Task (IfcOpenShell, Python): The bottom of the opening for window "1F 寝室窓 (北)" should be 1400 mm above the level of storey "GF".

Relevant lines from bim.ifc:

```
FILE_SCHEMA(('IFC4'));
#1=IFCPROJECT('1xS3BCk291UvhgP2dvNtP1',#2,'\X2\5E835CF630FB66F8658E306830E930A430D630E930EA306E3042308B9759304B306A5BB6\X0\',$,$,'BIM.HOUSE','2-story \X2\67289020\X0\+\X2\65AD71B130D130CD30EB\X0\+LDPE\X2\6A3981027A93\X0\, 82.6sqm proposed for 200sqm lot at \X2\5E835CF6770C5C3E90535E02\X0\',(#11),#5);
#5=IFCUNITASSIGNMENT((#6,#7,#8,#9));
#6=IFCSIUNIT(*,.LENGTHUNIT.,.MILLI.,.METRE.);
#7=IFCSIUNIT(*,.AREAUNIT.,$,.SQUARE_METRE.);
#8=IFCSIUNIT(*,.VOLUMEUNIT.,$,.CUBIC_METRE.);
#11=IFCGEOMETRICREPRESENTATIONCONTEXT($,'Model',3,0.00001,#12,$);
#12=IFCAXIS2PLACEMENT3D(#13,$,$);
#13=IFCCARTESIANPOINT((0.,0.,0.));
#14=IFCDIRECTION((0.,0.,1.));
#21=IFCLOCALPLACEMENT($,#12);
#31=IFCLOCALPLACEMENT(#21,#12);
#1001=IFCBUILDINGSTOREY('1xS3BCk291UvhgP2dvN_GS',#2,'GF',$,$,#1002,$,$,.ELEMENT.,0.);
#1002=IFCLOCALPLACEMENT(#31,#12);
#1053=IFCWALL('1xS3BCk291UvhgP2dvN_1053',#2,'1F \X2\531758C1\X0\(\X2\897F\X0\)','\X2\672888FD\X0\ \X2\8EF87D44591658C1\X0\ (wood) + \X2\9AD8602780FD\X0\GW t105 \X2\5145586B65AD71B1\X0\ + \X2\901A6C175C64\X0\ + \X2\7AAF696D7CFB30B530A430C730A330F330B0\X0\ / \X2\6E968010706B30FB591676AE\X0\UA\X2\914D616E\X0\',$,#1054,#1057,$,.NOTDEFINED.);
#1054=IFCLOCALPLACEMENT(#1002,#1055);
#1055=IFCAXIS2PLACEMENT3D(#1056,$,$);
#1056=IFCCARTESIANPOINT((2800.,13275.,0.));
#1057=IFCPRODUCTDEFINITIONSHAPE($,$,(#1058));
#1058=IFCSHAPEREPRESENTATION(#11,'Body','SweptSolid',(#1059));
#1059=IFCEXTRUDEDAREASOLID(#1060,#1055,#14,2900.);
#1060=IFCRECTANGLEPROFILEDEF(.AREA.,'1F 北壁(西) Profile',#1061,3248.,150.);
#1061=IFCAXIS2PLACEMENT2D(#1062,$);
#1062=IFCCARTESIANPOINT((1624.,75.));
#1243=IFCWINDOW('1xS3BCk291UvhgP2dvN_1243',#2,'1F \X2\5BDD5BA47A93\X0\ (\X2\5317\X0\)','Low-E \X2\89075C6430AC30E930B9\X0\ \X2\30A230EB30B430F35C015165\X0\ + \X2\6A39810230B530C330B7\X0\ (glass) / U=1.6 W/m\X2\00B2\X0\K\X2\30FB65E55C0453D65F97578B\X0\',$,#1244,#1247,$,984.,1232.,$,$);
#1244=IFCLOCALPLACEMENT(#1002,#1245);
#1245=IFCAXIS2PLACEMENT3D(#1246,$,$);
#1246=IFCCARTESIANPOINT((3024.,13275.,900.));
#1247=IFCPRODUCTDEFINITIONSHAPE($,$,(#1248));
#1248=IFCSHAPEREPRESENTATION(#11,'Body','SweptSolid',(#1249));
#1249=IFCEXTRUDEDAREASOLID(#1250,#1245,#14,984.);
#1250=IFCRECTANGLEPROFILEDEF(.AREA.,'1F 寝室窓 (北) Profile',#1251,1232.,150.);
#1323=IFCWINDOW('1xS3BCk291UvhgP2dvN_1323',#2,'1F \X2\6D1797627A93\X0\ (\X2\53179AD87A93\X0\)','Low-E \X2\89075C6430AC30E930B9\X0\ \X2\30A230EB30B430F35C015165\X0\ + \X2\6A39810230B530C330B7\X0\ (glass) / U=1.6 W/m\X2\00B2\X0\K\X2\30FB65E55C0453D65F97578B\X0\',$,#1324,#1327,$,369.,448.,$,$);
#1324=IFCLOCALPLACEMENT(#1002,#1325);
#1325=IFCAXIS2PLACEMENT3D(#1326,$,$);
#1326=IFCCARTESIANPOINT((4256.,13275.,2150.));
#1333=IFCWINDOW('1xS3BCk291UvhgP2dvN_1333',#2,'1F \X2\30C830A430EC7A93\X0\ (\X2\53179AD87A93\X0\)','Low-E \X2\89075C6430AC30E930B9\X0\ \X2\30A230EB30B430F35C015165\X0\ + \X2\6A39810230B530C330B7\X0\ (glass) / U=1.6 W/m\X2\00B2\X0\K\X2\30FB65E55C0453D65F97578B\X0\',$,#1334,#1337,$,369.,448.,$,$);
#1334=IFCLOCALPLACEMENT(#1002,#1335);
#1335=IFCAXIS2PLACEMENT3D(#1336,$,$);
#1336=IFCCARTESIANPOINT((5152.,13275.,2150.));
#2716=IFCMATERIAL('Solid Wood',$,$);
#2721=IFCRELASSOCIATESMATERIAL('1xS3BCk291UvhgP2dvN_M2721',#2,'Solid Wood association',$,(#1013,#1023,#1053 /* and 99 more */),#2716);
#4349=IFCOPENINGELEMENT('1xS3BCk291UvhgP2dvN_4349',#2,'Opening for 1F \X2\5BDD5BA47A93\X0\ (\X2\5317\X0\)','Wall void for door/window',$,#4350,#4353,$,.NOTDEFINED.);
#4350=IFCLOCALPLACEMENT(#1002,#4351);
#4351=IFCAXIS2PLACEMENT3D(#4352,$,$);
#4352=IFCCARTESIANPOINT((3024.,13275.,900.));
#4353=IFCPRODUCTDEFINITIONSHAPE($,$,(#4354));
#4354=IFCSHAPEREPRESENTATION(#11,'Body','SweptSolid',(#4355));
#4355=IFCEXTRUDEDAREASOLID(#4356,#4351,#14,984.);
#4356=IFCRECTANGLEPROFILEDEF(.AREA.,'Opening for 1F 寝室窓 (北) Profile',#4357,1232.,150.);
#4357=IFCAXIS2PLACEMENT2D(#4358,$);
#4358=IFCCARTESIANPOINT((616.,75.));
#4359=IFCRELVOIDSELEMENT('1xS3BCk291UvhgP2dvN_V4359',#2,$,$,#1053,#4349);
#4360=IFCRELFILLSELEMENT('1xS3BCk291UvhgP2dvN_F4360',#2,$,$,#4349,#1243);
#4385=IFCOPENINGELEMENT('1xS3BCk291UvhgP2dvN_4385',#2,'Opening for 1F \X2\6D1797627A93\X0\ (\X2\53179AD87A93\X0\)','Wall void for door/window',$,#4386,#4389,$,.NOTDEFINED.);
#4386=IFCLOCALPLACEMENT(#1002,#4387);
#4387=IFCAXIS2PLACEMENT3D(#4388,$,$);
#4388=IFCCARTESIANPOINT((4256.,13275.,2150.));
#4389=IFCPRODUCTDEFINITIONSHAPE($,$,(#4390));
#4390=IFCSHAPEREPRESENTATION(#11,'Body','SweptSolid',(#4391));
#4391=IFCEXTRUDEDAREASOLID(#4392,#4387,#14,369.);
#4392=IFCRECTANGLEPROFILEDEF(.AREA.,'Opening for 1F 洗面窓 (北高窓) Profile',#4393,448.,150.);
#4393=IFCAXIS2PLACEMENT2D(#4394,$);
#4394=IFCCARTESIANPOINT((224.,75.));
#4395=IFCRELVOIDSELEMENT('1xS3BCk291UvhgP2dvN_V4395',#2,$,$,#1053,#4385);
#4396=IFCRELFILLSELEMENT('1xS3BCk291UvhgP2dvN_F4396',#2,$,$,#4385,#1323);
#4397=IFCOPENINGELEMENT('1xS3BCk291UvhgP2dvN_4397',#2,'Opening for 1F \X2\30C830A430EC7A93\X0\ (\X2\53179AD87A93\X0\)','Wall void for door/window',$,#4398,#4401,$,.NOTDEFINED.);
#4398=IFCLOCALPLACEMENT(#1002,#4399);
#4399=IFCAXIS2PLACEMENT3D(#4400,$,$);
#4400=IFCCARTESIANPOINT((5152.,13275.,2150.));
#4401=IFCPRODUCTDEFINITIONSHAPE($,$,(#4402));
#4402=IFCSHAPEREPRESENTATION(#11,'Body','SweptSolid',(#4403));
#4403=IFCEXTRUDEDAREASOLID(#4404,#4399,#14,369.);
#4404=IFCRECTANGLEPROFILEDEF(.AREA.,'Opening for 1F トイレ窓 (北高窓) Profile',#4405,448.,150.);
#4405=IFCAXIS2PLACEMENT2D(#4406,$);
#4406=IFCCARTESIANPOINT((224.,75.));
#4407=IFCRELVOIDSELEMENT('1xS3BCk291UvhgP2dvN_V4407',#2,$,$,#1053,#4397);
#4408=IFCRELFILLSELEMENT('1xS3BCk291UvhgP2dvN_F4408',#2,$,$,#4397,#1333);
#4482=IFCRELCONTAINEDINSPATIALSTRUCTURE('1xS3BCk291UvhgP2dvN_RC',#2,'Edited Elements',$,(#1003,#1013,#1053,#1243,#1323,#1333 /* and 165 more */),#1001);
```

```python
import numpy as np
import ifcopenshell
import ifcopenshell.api.geometry
import ifcopenshell.geom
import ifcopenshell.util.element
import ifcopenshell.util.placement
import ifcopenshell.util.shape
import ifcopenshell.util.unit

model = ifcopenshell.open("bim.ifc")
unit_scale = ifcopenshell.util.unit.calculate_unit_scale(model)

window = model.by_guid("1xS3BCk291UvhgP2dvN_1243")
opening = window.FillsVoids[0].RelatingOpeningElement
storey = ifcopenshell.util.element.get_container(window, ifc_class="IfcBuildingStorey")
level = ifcopenshell.util.placement.get_local_placement(storey.ObjectPlacement)[2, 3]

# The opening's origin need not be at the sill, so measure its lowest point.
shape = ifcopenshell.geom.create_shape(ifcopenshell.geom.settings(), opening)
bottom = ifcopenshell.util.shape.get_shape_bottom_elevation(shape, shape.geometry) / unit_scale
dz = level + 1400.0 - bottom

shift = np.array([0.0, 0.0, dz])
# The window is not placed relative to its opening, so move both.
for product in (opening, window):
    matrix = ifcopenshell.util.placement.get_local_placement(product.ObjectPlacement)
    matrix[:3, 3] += shift
    ifcopenshell.api.geometry.edit_object_placement(model, product=product, matrix=matrix, is_si=False)

print(f"moved by {dz * unit_scale:+.3f} m")

model.write("bim_updated.ifc")
```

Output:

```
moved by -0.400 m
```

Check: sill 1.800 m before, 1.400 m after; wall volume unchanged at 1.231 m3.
